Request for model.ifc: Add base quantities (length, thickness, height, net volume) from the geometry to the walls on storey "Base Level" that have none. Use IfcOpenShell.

First a look at what the model holds.

```python
import ifcopenshell
import ifcopenshell.util.element
import ifcopenshell.util.unit

model = ifcopenshell.open("model.ifc")
print(model.schema)
for unit_type in ("LENGTHUNIT", "AREAUNIT", "VOLUMEUNIT"):
    print(unit_type, ifcopenshell.util.unit.calculate_unit_scale(model, unit_type))
storey = next(s for s in model.by_type("IfcBuildingStorey") if s.Name == "Base Level")
walls = [e for e in ifcopenshell.util.element.get_decomposition(storey) if e.is_a("IfcWall")]
for e in sorted(walls, key=lambda e: e.id()):
    print(e.id(), e.is_a(), e.Name, list(ifcopenshell.util.element.get_psets(e, qtos_only=True)), sep=" | ")
```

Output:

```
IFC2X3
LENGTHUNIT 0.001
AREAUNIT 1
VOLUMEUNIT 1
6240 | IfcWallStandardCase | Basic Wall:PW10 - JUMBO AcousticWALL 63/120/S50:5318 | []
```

```python
import ifcopenshell
import ifcopenshell.api.pset
import ifcopenshell.geom
import ifcopenshell.util.element
import ifcopenshell.util.shape
import ifcopenshell.util.unit

model = ifcopenshell.open("model.ifc")
unit_scale = ifcopenshell.util.unit.calculate_unit_scale(model)
volume_scale = ifcopenshell.util.unit.calculate_unit_scale(model, "VOLUMEUNIT")
settings = ifcopenshell.geom.settings()

storey = next(s for s in model.by_type("IfcBuildingStorey") if s.Name == "Base Level")
walls = [e for e in ifcopenshell.util.element.get_decomposition(storey) if e.is_a("IfcWall")]

for e in sorted(walls, key=lambda e: e.id()):
    if ifcopenshell.util.element.get_psets(e, qtos_only=True, should_inherit=False):
        continue
    # Geometry comes back in metres, in the element's own axes.
    shape = ifcopenshell.geom.create_shape(settings, e)
    values = {
        "Length": ifcopenshell.util.shape.get_x(shape.geometry) / unit_scale,
        "Width": ifcopenshell.util.shape.get_y(shape.geometry) / unit_scale,
        "Height": ifcopenshell.util.shape.get_z(shape.geometry) / unit_scale,
        "NetVolume": ifcopenshell.util.shape.get_volume(shape.geometry) / volume_scale,
    }
    qto = ifcopenshell.api.pset.add_qto(model, product=e, name="BaseQuantities")
    ifcopenshell.api.pset.edit_qto(model, qto=qto, properties=values)
    print(e.id(), {k: round(v, 3) for k, v in values.items()})

model.write("model-out.ifc")
```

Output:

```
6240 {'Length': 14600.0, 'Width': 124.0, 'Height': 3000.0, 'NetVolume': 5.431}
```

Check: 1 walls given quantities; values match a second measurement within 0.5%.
